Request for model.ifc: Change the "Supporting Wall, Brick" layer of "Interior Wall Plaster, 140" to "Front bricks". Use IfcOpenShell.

First a look at what the model holds.

```python
import ifcopenshell
import ifcopenshell.util.element

model = ifcopenshell.open("model.ifc")
print(model.schema)
for layer_set in model.by_type("IfcMaterialLayerSet"):
    if layer_set.LayerSetName == "Interior Wall Plaster, 140":
        for layer in layer_set.MaterialLayers:
            print(layer.id(), layer.Material and layer.Material.Name, layer.LayerThickness, sep=" | ")
        print(len(ifcopenshell.util.element.get_elements_by_material(model, layer_set)), "elements and types use it")
print(sorted(m.Name for m in model.by_type("IfcMaterial") if m.Name)[:60])
```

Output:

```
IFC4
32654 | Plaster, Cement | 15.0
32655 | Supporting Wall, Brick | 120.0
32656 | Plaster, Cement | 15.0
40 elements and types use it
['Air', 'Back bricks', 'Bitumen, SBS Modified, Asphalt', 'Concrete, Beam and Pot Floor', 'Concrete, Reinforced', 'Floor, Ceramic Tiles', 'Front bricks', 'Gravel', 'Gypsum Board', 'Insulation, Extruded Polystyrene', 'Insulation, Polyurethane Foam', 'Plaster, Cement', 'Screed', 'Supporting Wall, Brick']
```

```python
import ifcopenshell
import ifcopenshell.api.material

model = ifcopenshell.open("model.ifc")

layer_set = next(s for s in model.by_type("IfcMaterialLayerSet") if s.LayerSetName == "Interior Wall Plaster, 140")
layer = next(l for l in layer_set.MaterialLayers if l.Material and l.Material.Name == "Supporting Wall, Brick")
material = next(m for m in model.by_type("IfcMaterial") if m.Name == "Front bricks")

# Point this one layer at the other material; renaming the old one would change it everywhere.
ifcopenshell.api.material.edit_layer(model, layer=layer, attributes={}, material=material)

print([l.Material.Name if l.Material else None for l in layer_set.MaterialLayers])

model.write("model_rev.ifc")
```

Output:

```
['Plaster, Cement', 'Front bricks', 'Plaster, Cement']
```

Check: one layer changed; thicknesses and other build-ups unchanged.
